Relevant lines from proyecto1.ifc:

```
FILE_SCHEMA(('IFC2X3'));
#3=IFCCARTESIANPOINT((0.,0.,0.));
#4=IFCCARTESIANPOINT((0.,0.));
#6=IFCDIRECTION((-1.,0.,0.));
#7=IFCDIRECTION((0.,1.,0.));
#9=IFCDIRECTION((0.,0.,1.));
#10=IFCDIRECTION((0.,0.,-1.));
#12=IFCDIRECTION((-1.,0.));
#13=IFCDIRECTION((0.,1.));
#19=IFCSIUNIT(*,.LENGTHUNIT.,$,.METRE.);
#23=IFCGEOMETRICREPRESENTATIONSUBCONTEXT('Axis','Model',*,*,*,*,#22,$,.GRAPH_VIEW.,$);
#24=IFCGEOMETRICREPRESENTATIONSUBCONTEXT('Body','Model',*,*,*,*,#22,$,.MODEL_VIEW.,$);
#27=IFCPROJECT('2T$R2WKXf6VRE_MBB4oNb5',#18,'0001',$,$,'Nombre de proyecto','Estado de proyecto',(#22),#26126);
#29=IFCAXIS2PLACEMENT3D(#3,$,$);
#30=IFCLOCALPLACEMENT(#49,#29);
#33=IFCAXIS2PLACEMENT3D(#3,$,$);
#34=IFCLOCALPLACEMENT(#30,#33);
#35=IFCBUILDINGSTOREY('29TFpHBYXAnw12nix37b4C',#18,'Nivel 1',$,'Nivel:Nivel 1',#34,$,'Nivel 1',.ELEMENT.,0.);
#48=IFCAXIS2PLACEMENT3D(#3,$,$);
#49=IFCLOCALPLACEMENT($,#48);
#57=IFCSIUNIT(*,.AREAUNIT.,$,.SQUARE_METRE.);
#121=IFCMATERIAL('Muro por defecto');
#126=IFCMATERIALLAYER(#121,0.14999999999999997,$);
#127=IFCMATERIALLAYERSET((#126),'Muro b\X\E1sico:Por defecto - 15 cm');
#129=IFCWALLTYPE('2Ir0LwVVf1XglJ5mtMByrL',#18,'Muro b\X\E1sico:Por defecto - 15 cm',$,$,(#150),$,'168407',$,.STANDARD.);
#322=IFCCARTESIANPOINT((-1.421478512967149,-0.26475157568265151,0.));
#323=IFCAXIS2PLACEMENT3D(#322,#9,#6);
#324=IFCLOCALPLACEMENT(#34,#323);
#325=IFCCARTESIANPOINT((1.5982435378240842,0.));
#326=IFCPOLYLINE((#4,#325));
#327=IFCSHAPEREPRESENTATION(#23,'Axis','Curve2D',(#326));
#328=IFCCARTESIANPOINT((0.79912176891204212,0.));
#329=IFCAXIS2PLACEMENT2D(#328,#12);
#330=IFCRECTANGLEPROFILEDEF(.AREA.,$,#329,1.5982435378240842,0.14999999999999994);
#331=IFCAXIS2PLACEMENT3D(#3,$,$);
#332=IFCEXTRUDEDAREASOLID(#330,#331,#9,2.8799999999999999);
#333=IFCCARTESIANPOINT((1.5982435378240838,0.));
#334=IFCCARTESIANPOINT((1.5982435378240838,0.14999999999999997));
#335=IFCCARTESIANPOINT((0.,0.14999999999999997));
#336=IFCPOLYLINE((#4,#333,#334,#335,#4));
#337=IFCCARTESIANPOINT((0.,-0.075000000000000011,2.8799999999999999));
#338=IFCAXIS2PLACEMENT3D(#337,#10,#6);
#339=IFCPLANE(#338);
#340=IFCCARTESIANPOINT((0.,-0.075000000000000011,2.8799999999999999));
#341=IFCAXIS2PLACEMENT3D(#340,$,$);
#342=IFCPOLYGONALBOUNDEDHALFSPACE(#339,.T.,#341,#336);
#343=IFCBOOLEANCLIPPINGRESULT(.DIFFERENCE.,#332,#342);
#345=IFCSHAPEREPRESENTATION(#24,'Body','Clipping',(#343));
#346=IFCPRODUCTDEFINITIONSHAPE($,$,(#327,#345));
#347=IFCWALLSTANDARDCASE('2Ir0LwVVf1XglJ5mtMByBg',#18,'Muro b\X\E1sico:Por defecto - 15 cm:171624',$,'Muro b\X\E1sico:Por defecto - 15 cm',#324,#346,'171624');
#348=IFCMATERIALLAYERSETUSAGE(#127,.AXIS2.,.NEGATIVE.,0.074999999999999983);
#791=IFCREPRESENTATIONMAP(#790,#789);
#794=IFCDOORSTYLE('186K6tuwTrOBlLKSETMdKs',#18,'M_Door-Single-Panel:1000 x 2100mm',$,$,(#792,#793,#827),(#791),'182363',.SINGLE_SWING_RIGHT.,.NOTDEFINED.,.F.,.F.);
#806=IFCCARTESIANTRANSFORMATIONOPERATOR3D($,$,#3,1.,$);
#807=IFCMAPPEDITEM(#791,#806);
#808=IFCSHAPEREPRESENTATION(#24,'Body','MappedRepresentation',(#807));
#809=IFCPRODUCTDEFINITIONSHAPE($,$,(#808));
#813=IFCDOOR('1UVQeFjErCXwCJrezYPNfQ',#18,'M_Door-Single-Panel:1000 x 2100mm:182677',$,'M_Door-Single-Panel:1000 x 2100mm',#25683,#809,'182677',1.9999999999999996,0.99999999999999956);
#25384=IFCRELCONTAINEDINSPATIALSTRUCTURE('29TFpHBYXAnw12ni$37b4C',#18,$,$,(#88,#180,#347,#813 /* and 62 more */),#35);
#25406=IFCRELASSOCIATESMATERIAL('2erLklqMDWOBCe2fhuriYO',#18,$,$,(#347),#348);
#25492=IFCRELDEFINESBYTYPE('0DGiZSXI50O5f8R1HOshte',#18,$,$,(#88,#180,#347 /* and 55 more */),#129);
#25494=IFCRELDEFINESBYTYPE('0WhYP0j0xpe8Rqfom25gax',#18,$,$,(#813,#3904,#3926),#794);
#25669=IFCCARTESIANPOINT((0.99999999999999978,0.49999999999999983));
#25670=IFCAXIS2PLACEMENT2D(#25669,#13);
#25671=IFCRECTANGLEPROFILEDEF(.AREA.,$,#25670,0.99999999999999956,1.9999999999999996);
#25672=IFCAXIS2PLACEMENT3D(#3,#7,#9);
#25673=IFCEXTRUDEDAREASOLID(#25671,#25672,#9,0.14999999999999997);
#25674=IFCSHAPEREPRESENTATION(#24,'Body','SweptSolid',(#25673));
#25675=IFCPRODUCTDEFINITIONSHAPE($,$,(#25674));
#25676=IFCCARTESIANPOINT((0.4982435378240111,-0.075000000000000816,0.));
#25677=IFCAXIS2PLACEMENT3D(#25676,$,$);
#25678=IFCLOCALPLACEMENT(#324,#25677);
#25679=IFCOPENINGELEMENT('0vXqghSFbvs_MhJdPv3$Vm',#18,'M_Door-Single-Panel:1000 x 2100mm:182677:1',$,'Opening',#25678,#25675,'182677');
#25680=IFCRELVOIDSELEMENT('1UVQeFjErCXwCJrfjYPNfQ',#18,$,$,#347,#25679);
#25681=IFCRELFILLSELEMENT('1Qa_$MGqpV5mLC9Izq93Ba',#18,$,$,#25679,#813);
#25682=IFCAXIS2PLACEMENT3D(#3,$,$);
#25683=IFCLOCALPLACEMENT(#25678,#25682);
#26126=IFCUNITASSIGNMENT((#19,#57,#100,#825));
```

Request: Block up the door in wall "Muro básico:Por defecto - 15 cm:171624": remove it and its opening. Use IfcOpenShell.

```python
import ifcopenshell
import ifcopenshell.api.feature
import ifcopenshell.api.root
import ifcopenshell.geom
import ifcopenshell.util.shape

model = ifcopenshell.open("proyecto1.ifc")
settings = ifcopenshell.geom.settings()


def volume(element):
    """Net volume in cubic metres, openings subtracted."""
    shape = ifcopenshell.geom.create_shape(settings, element)
    return ifcopenshell.util.shape.get_volume(shape.geometry)


door = model.by_id(813)
opening = door.FillsVoids[0].RelatingOpeningElement
wall = opening.VoidsElements[0].RelatingBuildingElement
before = volume(wall)

ifcopenshell.api.root.remove_product(model, product=door)
ifcopenshell.api.feature.remove_feature(model, feature=opening)

after = volume(wall)

print(f"wall volume {before:.3f} -> {after:.3f} m3")

model.write("proyecto1_updated.ifc")
```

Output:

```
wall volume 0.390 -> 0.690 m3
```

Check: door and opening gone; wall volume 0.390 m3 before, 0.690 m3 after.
